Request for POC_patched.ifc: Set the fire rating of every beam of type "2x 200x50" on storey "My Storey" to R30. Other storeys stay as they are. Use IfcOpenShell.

First a look at what the model holds.

```python
import ifcopenshell
import ifcopenshell.util.element

model = ifcopenshell.open("POC_patched.ifc")
print(model.schema)
storey = next(s for s in model.by_type("IfcBuildingStorey") if s.Name == "My Storey")
beams = [e for e in ifcopenshell.util.element.get_decomposition(storey) if e.is_a("IfcBeam")]
seen = {}
for e in beams:
    element_type = ifcopenshell.util.element.get_type(e)
    key = (element_type.Name if element_type != e and element_type else None, ifcopenshell.util.element.get_pset(e, "Pset_BeamCommon", "FireRating"))
    seen[key] = seen.get(key, 0) + 1
for (name, value), count in sorted(seen.items(), key=str):
    print(count, "x", name, "|", value)
```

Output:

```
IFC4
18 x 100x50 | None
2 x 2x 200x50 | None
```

```python
import ifcopenshell
import ifcopenshell.api.pset
import ifcopenshell.util.element

model = ifcopenshell.open("POC_patched.ifc")

storey = next(s for s in model.by_type("IfcBuildingStorey") if s.Name == "My Storey")
beams = [e for e in ifcopenshell.util.element.get_decomposition(storey) if e.is_a("IfcBeam")]

count = 0
for e in beams:
    element_type = ifcopenshell.util.element.get_type(e)
    if element_type in (None, e) or element_type.Name != "2x 200x50":
        continue
    # add_pset returns the element's existing set when there is one.
    pset = ifcopenshell.api.pset.add_pset(model, product=e, name="Pset_BeamCommon")
    ifcopenshell.api.pset.edit_pset(model, pset=pset, properties={"FireRating": "R30"})
    count += 1

print(count, "beams updated")

model.write("POC_patched_edited.ifc")
```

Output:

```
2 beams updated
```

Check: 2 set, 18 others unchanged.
